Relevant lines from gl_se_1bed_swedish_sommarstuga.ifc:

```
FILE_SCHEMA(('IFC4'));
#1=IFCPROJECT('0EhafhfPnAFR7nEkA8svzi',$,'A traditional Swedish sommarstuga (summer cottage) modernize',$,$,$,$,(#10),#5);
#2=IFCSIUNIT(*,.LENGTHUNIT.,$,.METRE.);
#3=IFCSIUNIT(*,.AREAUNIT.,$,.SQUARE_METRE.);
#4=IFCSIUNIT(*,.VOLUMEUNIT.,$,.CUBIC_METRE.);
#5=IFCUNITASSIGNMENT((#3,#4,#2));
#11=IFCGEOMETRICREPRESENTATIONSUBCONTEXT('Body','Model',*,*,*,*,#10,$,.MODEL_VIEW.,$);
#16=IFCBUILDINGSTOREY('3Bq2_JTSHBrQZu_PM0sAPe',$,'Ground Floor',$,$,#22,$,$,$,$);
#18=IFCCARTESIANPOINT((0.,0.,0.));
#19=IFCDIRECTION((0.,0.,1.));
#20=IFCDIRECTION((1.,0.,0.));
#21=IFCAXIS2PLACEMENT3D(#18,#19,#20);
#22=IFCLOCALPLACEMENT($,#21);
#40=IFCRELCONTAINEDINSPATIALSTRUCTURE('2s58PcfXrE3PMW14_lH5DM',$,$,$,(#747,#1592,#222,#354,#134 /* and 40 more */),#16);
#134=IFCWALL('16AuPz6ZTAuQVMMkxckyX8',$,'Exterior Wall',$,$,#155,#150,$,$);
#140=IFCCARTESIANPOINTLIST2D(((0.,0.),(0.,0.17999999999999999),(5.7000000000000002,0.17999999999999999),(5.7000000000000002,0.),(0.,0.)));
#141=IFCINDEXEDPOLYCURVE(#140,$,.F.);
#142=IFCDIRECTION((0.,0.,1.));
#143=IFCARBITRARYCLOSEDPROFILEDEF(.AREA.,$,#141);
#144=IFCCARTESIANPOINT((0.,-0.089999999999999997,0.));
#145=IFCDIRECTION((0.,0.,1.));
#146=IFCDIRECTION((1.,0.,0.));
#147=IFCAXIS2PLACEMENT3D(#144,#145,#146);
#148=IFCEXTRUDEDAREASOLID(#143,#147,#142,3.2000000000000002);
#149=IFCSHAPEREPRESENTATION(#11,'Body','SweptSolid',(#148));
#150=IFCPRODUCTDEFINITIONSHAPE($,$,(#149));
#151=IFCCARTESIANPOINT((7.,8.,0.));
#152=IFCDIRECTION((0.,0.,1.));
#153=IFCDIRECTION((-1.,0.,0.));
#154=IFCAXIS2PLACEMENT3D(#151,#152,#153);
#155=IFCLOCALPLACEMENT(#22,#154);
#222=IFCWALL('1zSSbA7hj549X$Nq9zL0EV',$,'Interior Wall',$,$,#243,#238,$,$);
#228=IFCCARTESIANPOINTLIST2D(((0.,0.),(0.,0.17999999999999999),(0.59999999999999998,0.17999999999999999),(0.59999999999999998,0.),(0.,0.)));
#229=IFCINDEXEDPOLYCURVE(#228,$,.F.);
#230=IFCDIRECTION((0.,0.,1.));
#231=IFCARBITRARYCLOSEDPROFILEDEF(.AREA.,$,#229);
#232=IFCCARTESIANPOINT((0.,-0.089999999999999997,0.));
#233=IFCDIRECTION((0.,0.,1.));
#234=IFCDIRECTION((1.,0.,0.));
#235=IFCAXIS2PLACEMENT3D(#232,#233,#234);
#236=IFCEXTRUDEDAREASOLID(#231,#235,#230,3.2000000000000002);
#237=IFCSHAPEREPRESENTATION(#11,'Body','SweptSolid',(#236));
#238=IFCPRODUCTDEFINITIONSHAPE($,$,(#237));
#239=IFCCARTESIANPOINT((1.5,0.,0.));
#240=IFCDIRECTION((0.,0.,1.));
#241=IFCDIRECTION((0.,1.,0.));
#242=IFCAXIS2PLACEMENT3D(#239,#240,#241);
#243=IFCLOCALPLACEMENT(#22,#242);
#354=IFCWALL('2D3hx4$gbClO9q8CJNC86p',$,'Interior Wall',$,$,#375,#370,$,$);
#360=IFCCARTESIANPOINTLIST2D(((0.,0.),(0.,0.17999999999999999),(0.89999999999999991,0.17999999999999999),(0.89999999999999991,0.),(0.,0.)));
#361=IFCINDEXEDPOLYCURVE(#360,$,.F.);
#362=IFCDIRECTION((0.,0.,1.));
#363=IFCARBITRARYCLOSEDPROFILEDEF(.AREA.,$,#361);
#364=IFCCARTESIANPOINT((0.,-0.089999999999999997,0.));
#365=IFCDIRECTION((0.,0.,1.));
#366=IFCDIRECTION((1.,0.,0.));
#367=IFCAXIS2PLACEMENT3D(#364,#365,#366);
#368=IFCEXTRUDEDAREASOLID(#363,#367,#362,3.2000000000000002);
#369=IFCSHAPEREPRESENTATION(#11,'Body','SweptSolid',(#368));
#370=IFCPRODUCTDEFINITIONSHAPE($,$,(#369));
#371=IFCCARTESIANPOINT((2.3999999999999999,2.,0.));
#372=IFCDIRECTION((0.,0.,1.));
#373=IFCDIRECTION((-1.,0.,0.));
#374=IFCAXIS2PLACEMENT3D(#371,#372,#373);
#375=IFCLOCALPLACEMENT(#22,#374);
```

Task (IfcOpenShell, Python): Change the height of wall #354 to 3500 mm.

```python
import ifcopenshell
import ifcopenshell.geom
import ifcopenshell.util.representation
import ifcopenshell.util.shape

model = ifcopenshell.open("gl_se_1bed_swedish_sommarstuga.ifc")
settings = ifcopenshell.geom.settings()


def volume(element):
    """Net volume in cubic metres, openings subtracted."""
    shape = ifcopenshell.geom.create_shape(settings, element)
    return ifcopenshell.util.shape.get_volume(shape.geometry)


wall = model.by_guid("2D3hx4$gbClO9q8CJNC86p")
before = volume(wall)

body = ifcopenshell.util.representation.get_representation(wall, "Model", "Body")
solid = body.Items[0]
old_height = solid.Depth
solid.Depth = 3.5
after = volume(wall)

print(f"height {old_height:g} -> {solid.Depth:g}, volume {before:.3f} -> {after:.3f} m3")

model.write("gl_se_1bed_swedish_sommarstuga_rev.ifc")
```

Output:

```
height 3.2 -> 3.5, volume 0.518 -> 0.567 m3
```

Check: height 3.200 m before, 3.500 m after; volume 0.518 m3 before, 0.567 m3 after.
